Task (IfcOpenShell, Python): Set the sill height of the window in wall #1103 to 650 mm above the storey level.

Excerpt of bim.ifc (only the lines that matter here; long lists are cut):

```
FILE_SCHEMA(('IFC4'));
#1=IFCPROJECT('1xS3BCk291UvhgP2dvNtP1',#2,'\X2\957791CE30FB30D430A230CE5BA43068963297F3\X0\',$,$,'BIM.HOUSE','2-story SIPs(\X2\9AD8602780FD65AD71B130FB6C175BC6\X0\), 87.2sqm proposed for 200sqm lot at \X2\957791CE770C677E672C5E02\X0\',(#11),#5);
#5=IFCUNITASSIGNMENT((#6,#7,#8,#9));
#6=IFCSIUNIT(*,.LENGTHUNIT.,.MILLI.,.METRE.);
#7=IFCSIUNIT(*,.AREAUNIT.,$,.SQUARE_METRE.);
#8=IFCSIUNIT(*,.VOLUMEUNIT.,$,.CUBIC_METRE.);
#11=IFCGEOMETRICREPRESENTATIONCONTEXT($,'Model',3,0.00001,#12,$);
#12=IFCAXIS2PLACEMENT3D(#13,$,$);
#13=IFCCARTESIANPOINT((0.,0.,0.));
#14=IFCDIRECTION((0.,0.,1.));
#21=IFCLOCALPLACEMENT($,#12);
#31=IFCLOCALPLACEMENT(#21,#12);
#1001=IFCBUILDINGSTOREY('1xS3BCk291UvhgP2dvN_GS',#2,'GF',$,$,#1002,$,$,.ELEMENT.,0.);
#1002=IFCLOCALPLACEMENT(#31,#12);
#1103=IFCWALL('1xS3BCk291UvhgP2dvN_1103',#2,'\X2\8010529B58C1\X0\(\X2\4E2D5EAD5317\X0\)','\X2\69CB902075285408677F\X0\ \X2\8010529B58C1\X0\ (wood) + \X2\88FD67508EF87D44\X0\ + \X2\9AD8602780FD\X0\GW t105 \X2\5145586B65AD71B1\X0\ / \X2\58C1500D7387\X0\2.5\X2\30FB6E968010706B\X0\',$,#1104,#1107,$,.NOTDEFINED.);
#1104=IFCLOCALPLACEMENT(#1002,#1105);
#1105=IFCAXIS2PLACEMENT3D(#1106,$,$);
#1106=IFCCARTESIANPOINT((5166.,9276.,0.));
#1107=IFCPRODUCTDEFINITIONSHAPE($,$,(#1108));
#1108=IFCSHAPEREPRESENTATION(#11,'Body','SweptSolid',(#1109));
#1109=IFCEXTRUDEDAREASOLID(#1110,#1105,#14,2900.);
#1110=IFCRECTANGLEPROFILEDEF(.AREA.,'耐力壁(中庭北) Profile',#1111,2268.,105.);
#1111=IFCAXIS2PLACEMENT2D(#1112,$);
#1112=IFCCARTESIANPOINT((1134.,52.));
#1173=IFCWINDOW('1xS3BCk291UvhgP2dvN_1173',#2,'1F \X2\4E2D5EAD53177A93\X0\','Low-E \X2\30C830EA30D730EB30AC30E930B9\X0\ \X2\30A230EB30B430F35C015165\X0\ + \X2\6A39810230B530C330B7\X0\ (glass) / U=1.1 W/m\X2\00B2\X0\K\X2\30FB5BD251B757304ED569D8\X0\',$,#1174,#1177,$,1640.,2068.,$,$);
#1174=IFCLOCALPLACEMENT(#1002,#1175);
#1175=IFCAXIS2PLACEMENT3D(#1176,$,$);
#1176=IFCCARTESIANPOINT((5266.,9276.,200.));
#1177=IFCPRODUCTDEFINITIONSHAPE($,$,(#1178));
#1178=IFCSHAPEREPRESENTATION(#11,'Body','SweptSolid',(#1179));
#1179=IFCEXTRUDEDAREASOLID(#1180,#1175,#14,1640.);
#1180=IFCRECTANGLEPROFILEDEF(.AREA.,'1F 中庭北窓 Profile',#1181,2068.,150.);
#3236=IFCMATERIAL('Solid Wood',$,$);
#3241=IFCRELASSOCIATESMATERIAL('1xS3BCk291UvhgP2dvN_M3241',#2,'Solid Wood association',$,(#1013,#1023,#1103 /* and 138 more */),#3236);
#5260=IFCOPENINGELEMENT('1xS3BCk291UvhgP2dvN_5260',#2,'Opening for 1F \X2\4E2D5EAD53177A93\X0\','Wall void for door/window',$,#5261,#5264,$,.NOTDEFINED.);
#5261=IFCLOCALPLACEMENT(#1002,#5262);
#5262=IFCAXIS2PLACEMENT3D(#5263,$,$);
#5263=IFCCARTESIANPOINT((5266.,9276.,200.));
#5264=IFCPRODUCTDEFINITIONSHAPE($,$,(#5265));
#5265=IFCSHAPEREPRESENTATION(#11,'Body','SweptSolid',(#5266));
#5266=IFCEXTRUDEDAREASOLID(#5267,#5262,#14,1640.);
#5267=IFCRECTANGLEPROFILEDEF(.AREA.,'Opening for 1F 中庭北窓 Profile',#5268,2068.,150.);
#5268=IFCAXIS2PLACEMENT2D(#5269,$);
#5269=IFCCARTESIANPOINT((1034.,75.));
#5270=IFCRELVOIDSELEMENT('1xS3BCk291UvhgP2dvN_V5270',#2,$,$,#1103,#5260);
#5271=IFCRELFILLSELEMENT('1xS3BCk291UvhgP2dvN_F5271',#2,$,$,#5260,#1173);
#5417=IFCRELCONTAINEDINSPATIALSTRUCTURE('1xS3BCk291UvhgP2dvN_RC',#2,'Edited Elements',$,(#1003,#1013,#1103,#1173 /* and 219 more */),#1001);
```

```python
import numpy as np
import ifcopenshell
import ifcopenshell.api.geometry
import ifcopenshell.geom
import ifcopenshell.util.element
import ifcopenshell.util.placement
import ifcopenshell.util.shape
import ifcopenshell.util.unit

model = ifcopenshell.open("bim.ifc")
unit_scale = ifcopenshell.util.unit.calculate_unit_scale(model)

window = model.by_guid("1xS3BCk291UvhgP2dvN_1173")
opening = window.FillsVoids[0].RelatingOpeningElement
storey = ifcopenshell.util.element.get_container(window, ifc_class="IfcBuildingStorey")
level = ifcopenshell.util.placement.get_local_placement(storey.ObjectPlacement)[2, 3]

# The opening's origin need not be at the sill, so measure its lowest point.
shape = ifcopenshell.geom.create_shape(ifcopenshell.geom.settings(), opening)
bottom = ifcopenshell.util.shape.get_shape_bottom_elevation(shape, shape.geometry) / unit_scale
dz = level + 0.65 / unit_scale - bottom

shift = np.array([0.0, 0.0, dz])
# The window is not placed relative to its opening, so move both.
for product in (opening, window):
    matrix = ifcopenshell.util.placement.get_local_placement(product.ObjectPlacement)
    matrix[:3, 3] += shift
    ifcopenshell.api.geometry.edit_object_placement(model, product=product, matrix=matrix, is_si=False)

print(f"moved by {dz * unit_scale:+.3f} m")

model.write("bim-out.ifc")
```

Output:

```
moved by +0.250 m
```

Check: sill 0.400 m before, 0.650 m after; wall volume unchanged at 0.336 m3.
